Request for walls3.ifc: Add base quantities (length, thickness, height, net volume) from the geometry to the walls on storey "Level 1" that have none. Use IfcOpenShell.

First a look at what the model holds.

```python
import ifcopenshell
import ifcopenshell.util.element
import ifcopenshell.util.unit

model = ifcopenshell.open("walls3.ifc")
print(model.schema)
for unit_type in ("LENGTHUNIT", "AREAUNIT", "VOLUMEUNIT"):
    print(unit_type, ifcopenshell.util.unit.calculate_unit_scale(model, unit_type))
storey = next(s for s in model.by_type("IfcBuildingStorey") if s.Name == "Level 1")
walls = [e for e in ifcopenshell.util.element.get_decomposition(storey) if e.is_a("IfcWall")]
for e in sorted(walls, key=lambda e: e.id()):
    print(e.id(), e.is_a(), e.Name, list(ifcopenshell.util.element.get_psets(e, qtos_only=True)), sep=" | ")
```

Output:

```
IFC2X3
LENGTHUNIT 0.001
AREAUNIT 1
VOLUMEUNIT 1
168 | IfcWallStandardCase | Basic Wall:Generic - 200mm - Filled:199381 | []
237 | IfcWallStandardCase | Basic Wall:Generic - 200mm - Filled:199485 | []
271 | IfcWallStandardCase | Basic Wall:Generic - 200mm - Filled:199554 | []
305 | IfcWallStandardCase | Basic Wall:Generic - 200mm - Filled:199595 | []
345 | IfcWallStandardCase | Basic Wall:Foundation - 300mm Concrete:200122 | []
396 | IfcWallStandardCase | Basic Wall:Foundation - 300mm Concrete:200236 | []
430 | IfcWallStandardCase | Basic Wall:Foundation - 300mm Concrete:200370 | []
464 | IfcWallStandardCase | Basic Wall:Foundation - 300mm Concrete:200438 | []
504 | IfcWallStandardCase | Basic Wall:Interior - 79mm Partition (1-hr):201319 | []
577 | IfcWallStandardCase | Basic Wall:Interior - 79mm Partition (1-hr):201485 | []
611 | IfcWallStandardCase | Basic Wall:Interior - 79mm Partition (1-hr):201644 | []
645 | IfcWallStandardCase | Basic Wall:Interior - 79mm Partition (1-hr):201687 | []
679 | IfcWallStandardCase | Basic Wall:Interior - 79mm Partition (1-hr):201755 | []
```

```python
import ifcopenshell
import ifcopenshell.api.pset
import ifcopenshell.geom
import ifcopenshell.util.element
import ifcopenshell.util.shape
import ifcopenshell.util.unit

model = ifcopenshell.open("walls3.ifc")
unit_scale = ifcopenshell.util.unit.calculate_unit_scale(model)
volume_scale = ifcopenshell.util.unit.calculate_unit_scale(model, "VOLUMEUNIT")
settings = ifcopenshell.geom.settings()

storey = next(s for s in model.by_type("IfcBuildingStorey") if s.Name == "Level 1")
walls = [e for e in ifcopenshell.util.element.get_decomposition(storey) if e.is_a("IfcWall")]

for e in sorted(walls, key=lambda e: e.id()):
    if ifcopenshell.util.element.get_psets(e, qtos_only=True, should_inherit=False):
        continue
    # Geometry comes back in metres, in the element's own axes.
    shape = ifcopenshell.geom.create_shape(settings, e)
    values = {
        "Length": ifcopenshell.util.shape.get_x(shape.geometry) / unit_scale,
        "Width": ifcopenshell.util.shape.get_y(shape.geometry) / unit_scale,
        "Height": ifcopenshell.util.shape.get_z(shape.geometry) / unit_scale,
        "NetVolume": ifcopenshell.util.shape.get_volume(shape.geometry) / volume_scale,
    }
    qto = ifcopenshell.api.pset.add_qto(model, product=e, name="BaseQuantities")
    ifcopenshell.api.pset.edit_qto(model, qto=qto, properties=values)
    print(e.id(), {k: round(v, 3) for k, v in values.items()})

model.write("walls3_edited.ifc")
```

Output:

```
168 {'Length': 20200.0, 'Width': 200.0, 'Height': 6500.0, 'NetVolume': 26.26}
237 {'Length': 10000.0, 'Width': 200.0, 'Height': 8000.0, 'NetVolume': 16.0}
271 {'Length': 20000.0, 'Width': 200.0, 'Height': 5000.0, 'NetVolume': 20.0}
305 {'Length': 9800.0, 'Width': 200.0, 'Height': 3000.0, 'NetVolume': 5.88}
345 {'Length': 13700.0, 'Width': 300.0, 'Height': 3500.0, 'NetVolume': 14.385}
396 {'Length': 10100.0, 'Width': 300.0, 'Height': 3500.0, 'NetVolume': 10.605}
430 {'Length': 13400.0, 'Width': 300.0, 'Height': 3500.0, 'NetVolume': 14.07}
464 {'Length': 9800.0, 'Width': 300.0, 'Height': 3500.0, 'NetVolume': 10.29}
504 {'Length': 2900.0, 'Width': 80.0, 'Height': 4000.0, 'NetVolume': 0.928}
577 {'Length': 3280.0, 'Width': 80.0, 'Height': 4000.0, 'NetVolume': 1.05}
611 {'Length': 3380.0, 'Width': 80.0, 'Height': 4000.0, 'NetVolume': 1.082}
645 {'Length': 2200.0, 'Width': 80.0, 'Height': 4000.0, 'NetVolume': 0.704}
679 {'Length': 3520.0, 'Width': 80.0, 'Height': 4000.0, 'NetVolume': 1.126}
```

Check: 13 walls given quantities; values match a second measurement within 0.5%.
